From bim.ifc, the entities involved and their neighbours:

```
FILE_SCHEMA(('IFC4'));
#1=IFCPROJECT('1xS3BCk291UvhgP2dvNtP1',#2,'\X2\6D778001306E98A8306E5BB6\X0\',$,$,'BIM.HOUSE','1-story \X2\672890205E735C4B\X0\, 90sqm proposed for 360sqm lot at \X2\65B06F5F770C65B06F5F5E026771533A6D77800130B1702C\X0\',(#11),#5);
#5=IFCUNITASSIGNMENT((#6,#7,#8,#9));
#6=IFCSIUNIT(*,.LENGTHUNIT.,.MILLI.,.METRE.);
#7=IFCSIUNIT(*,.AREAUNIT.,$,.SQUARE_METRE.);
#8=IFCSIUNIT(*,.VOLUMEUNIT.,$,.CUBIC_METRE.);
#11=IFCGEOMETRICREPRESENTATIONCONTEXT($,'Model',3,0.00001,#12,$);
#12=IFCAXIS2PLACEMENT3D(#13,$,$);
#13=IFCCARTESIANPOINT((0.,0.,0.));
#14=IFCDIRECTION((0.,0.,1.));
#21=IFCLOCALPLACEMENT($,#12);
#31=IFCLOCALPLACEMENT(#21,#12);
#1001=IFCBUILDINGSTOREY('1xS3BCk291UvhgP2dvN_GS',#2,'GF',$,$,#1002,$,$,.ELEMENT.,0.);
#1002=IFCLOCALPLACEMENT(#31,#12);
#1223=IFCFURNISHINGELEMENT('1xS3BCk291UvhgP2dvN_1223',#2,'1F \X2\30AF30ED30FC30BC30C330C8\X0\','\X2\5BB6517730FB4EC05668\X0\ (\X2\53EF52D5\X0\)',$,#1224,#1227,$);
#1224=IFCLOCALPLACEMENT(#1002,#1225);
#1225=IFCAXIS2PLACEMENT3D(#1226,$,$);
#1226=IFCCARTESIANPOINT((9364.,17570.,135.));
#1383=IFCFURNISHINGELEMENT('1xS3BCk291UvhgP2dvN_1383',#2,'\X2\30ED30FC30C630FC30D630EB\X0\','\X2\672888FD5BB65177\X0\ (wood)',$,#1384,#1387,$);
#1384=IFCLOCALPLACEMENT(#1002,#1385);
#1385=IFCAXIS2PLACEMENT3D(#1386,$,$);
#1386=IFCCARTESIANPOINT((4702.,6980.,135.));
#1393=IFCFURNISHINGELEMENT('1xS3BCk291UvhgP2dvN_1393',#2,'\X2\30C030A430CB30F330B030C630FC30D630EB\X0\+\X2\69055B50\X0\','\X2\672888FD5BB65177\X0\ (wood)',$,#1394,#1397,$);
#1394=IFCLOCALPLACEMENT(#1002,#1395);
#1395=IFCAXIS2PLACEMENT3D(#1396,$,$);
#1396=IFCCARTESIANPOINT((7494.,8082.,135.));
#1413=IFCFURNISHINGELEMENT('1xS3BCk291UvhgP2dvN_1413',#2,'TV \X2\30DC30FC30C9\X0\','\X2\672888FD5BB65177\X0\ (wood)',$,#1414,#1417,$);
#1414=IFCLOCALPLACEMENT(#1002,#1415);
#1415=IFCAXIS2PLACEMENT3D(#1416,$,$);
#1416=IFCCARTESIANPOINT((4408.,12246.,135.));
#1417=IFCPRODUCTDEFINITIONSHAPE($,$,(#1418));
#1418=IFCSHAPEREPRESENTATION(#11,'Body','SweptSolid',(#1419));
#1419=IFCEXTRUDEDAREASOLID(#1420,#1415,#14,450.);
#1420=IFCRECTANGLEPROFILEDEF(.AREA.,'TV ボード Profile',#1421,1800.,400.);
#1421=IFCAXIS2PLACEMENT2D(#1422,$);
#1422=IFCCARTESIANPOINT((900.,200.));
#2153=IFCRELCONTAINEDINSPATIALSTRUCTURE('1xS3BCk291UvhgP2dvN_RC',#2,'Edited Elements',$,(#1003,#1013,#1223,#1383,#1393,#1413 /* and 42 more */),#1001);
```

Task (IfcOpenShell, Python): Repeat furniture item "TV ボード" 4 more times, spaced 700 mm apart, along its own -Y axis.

```python
import ifcopenshell
import ifcopenshell.api.geometry
import ifcopenshell.api.root
import ifcopenshell.util.element
import ifcopenshell.util.placement

model = ifcopenshell.open("bim.ifc")


def reuse_history(source, copy):
    """copy_class also copies each property set's owner history, people and application; keep the originals."""
    for rel in copy.IsDefinedBy:
        if rel.is_a("IfcRelDefinesByProperties") and (history := rel.RelatingPropertyDefinition.OwnerHistory):
            rel.RelatingPropertyDefinition.OwnerHistory = source.OwnerHistory
            ifcopenshell.util.element.remove_deep2(model, history)


source = model.by_id(1413)
base = ifcopenshell.util.placement.get_local_placement(source.ObjectPlacement)
step = -base[:3, 1] * 700.0

for i in range(1, 5):
    copy = ifcopenshell.api.root.copy_class(model, product=source)
    copy.Representation = ifcopenshell.util.element.copy_deep(
        model, source.Representation, exclude=["IfcGeometricRepresentationContext", "IfcRepresentationMap"]
    )
    reuse_history(source, copy)
    matrix = base.copy()
    matrix[:3, 3] += i * step
    print("added at", matrix[:3, 3].round(3) + 0.0)
    ifcopenshell.api.geometry.edit_object_placement(model, product=copy, matrix=matrix, is_si=False)

model.write("bim_updated.ifc")
```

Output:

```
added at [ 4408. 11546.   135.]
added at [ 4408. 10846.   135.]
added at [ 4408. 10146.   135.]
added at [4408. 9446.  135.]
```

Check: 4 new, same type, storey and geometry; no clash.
